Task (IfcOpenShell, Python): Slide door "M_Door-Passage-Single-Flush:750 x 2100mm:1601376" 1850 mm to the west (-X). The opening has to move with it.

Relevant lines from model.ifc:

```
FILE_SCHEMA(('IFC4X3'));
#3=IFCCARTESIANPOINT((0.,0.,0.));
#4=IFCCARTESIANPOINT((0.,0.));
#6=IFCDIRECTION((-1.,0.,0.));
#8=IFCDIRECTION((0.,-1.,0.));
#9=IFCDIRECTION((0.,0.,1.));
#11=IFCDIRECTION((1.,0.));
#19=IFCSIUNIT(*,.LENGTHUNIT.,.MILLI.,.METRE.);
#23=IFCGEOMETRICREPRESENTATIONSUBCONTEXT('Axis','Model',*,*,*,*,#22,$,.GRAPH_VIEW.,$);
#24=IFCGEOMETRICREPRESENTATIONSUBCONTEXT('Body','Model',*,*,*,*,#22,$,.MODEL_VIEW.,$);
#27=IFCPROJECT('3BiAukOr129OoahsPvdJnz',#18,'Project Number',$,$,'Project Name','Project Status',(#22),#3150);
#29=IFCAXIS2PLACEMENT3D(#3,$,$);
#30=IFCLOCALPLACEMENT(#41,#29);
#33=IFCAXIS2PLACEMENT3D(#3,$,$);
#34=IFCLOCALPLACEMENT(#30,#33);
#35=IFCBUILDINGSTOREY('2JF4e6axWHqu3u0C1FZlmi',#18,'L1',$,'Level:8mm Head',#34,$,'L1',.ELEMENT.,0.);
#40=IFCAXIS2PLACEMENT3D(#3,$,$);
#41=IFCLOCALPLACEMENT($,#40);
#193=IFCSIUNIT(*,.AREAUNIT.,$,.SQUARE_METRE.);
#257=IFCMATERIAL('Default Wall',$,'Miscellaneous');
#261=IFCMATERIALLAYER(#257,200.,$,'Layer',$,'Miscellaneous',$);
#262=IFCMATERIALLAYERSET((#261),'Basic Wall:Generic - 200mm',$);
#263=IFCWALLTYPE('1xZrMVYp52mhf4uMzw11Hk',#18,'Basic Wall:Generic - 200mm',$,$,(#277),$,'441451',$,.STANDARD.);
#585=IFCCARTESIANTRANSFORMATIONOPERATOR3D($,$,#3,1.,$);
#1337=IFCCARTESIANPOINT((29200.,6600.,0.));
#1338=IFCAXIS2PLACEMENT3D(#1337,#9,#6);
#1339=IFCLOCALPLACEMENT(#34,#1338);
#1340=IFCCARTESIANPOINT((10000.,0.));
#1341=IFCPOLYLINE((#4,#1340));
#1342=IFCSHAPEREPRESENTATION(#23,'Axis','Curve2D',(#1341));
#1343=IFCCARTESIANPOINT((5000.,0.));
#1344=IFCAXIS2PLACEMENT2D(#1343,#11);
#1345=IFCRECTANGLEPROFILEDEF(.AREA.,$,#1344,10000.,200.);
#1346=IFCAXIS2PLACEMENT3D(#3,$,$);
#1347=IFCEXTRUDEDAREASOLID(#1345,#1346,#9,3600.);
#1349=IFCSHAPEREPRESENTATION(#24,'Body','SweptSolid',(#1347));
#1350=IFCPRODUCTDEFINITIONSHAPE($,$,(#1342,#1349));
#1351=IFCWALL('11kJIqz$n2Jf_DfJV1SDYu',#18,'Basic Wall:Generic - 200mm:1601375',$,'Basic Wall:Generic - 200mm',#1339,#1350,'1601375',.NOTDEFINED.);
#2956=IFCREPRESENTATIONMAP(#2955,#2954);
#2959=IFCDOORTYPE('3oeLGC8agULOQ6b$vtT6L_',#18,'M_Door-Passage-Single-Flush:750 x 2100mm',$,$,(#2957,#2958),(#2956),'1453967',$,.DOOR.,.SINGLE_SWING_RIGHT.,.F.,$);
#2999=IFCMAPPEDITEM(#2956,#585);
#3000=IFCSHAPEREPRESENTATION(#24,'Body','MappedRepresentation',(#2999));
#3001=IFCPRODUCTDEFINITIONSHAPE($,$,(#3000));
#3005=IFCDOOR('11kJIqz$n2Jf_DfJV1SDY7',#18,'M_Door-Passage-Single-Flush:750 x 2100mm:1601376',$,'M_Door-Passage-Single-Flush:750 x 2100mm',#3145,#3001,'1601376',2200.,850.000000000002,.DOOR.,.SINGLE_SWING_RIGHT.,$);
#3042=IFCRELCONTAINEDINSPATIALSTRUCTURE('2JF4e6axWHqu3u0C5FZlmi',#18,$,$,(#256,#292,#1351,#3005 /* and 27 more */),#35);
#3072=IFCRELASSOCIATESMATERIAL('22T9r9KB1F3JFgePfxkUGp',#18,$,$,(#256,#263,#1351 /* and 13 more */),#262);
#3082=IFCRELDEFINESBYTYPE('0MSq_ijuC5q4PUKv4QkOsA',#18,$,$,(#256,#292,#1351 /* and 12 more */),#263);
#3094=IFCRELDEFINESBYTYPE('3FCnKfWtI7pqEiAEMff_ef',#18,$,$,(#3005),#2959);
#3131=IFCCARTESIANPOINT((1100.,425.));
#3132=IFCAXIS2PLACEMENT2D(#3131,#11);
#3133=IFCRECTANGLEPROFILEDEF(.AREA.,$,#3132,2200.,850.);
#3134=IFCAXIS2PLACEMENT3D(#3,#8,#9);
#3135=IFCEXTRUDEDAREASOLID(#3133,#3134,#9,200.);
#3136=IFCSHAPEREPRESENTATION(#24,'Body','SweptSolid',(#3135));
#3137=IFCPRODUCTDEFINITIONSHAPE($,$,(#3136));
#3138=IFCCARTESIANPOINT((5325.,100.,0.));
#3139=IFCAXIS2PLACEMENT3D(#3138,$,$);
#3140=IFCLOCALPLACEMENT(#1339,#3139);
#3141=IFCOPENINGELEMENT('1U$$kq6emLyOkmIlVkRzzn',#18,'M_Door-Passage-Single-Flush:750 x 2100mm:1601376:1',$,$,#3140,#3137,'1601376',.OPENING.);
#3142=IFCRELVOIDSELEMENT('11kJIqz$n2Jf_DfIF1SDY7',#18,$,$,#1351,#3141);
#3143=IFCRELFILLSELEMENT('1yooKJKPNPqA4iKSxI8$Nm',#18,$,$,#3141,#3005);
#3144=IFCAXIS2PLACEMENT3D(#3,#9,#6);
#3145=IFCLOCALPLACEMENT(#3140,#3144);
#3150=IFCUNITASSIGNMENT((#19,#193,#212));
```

```python
import ifcopenshell
import ifcopenshell.api.geometry
import ifcopenshell.util.placement

model = ifcopenshell.open("model.ifc")

door = model.by_guid("11kJIqz$n2Jf_DfJV1SDY7")
opening = door.FillsVoids[0].RelatingOpeningElement
wall = opening.VoidsElements[0].RelatingBuildingElement

wall_matrix = ifcopenshell.util.placement.get_local_placement(wall.ObjectPlacement)
shift = wall_matrix[:3, 0] * 1850.0
before = ifcopenshell.util.placement.get_local_placement(door.ObjectPlacement)[:3, 3].copy()

# The door is placed relative to its opening, so it follows when the opening moves.
matrix = ifcopenshell.util.placement.get_local_placement(opening.ObjectPlacement)
matrix[:3, 3] += shift
ifcopenshell.api.geometry.edit_object_placement(
    model, product=opening, matrix=matrix, is_si=False, should_transform_children=True
)

after = ifcopenshell.util.placement.get_local_placement(door.ObjectPlacement)[:3, 3]
print("door moved by", (after - before).round(3) + 0.0)

model.write("model-out.ifc")
```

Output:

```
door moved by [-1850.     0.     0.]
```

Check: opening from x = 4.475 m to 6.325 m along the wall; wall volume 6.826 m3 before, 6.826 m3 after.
